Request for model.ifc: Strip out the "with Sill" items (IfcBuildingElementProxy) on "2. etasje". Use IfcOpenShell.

First a look at what the model holds.

```python
import ifcopenshell
import ifcopenshell.util.element

model = ifcopenshell.open("model.ifc")
print(model.schema)
storey = next(s for s in model.by_type("IfcBuildingStorey") if s.Name == "2. etasje")
proxies = [e for e in ifcopenshell.util.element.get_decomposition(storey) if e.is_a("IfcBuildingElementProxy")]
seen = {}
for e in proxies:
    element_type = ifcopenshell.util.element.get_type(e)
    name = element_type.Name if element_type not in (None, e) else None
    seen[name] = seen.get(name, 0) + 1
for name, count in sorted(seen.items(), key=str):
    print(count, "x", name)
```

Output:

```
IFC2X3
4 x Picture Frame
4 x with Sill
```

```python
import ifcopenshell
import ifcopenshell.api.root
import ifcopenshell.util.element

model = ifcopenshell.open("model.ifc")

storey = next(s for s in model.by_type("IfcBuildingStorey") if s.Name == "2. etasje")
proxies = [e for e in ifcopenshell.util.element.get_decomposition(storey) if e.is_a("IfcBuildingElementProxy")]
targets = [e for e in proxies if (t := ifcopenshell.util.element.get_type(e)) not in (None, e) and t.Name == "with Sill"]

for e in targets:
    ifcopenshell.api.root.remove_product(model, product=e)
print(len(targets), "removed")

model.write("model_v2.ifc")
```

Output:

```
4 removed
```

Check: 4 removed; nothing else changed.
